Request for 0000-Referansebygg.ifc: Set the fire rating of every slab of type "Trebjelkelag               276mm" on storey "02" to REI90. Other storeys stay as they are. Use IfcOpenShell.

First a look at what the model holds.

```python
import ifcopenshell
import ifcopenshell.util.element

model = ifcopenshell.open("0000-Referansebygg.ifc")
print(model.schema)
storey = next(s for s in model.by_type("IfcBuildingStorey") if s.Name == "02")
slabs = [e for e in ifcopenshell.util.element.get_decomposition(storey) if e.is_a("IfcSlab")]
seen = {}
for e in slabs:
    element_type = ifcopenshell.util.element.get_type(e)
    key = (element_type.Name if element_type != e and element_type else None, ifcopenshell.util.element.get_pset(e, "Pset_SlabCommon", "FireRating"))
    seen[key] = seen.get(key, 0) + 1
for (name, value), count in sorted(seen.items(), key=str):
    print(count, "x", name, "|", value)
```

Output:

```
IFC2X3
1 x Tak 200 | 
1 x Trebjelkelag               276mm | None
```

```python
import ifcopenshell
import ifcopenshell.api.pset
import ifcopenshell.util.element

model = ifcopenshell.open("0000-Referansebygg.ifc")

storey = next(s for s in model.by_type("IfcBuildingStorey") if s.Name == "02")
slabs = [e for e in ifcopenshell.util.element.get_decomposition(storey) if e.is_a("IfcSlab")]

count = 0
for e in slabs:
    element_type = ifcopenshell.util.element.get_type(e)
    if element_type in (None, e) or element_type.Name != "Trebjelkelag               276mm":
        continue
    # add_pset returns the element's existing set when there is one.
    pset = ifcopenshell.api.pset.add_pset(model, product=e, name="Pset_SlabCommon")
    ifcopenshell.api.pset.edit_pset(model, pset=pset, properties={"FireRating": "REI90"})
    count += 1

print(count, "slabs updated")

model.write("0000-Referansebygg-out.ifc")
```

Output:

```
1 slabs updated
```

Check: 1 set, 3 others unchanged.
